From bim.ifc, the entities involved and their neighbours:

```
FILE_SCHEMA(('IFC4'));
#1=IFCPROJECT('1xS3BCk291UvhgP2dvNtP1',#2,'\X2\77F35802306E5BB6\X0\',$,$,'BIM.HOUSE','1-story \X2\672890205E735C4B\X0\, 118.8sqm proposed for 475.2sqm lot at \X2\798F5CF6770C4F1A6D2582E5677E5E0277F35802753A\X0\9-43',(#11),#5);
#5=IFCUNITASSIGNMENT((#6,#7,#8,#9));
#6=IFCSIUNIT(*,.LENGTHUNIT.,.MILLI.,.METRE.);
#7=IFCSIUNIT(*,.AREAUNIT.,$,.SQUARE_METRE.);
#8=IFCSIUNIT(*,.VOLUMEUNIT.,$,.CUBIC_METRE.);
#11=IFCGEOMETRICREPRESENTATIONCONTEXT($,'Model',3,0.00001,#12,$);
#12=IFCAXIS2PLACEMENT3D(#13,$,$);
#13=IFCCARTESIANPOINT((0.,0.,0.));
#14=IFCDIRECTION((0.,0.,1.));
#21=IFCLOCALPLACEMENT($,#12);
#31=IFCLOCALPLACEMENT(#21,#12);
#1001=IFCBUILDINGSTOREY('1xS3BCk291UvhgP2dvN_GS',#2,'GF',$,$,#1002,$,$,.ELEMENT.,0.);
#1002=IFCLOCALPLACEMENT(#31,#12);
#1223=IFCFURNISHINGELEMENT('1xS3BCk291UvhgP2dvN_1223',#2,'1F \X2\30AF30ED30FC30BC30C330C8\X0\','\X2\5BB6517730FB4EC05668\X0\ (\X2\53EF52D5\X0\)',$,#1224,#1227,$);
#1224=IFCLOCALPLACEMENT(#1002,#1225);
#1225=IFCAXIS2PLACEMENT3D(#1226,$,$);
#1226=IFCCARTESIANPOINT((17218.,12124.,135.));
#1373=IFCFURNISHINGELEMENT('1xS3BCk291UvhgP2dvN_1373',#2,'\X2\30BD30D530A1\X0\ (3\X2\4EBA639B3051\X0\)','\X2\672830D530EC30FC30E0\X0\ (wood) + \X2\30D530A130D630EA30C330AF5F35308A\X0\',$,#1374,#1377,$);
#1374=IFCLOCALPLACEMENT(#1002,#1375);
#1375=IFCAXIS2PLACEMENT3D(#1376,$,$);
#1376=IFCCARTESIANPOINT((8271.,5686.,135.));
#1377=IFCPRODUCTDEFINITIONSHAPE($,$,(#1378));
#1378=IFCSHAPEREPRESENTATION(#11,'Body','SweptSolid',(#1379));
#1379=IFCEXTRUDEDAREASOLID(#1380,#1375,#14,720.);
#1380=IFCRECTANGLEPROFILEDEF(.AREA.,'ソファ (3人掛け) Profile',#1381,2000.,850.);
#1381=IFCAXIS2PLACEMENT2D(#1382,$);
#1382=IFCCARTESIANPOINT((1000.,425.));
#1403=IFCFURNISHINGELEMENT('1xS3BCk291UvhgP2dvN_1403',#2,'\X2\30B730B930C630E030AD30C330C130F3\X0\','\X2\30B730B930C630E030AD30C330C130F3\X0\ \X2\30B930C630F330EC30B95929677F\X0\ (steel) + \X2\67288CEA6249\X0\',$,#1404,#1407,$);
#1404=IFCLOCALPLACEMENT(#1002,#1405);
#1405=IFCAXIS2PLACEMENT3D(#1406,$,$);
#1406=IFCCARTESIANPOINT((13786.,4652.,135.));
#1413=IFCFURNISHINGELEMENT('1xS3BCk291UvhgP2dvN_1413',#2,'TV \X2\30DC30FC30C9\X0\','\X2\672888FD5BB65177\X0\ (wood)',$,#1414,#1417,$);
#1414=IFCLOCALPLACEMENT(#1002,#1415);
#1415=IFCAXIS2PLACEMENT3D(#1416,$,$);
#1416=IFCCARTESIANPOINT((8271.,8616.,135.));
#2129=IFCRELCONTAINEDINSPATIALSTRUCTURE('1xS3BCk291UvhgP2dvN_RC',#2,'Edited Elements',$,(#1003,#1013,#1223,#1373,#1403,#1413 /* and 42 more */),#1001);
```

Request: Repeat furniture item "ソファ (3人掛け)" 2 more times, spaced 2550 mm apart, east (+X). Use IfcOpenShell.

```python
import numpy as np
import ifcopenshell
import ifcopenshell.api.geometry
import ifcopenshell.api.root
import ifcopenshell.util.element
import ifcopenshell.util.placement
import ifcopenshell.util.unit

model = ifcopenshell.open("bim.ifc")
unit_scale = ifcopenshell.util.unit.calculate_unit_scale(model)


def reuse_history(source, copy):
    """copy_class also copies each property set's owner history, people and application; keep the originals."""
    for rel in copy.IsDefinedBy:
        if rel.is_a("IfcRelDefinesByProperties") and (history := rel.RelatingPropertyDefinition.OwnerHistory):
            rel.RelatingPropertyDefinition.OwnerHistory = source.OwnerHistory
            ifcopenshell.util.element.remove_deep2(model, history)


source = model.by_guid("1xS3BCk291UvhgP2dvN_1373")
base = ifcopenshell.util.placement.get_local_placement(source.ObjectPlacement)
step = np.array([1.0, 0.0, 0.0]) * 2.55 / unit_scale

for i in range(1, 3):
    copy = ifcopenshell.api.root.copy_class(model, product=source)
    copy.Representation = ifcopenshell.util.element.copy_deep(
        model, source.Representation, exclude=["IfcGeometricRepresentationContext", "IfcRepresentationMap"]
    )
    reuse_history(source, copy)
    matrix = base.copy()
    matrix[:3, 3] += i * step
    print("added at", matrix[:3, 3].round(3) + 0.0)
    ifcopenshell.api.geometry.edit_object_placement(model, product=copy, matrix=matrix, is_si=False)

model.write("bim_rev.ifc")
```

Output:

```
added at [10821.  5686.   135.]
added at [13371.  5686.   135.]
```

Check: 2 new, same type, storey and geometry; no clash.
